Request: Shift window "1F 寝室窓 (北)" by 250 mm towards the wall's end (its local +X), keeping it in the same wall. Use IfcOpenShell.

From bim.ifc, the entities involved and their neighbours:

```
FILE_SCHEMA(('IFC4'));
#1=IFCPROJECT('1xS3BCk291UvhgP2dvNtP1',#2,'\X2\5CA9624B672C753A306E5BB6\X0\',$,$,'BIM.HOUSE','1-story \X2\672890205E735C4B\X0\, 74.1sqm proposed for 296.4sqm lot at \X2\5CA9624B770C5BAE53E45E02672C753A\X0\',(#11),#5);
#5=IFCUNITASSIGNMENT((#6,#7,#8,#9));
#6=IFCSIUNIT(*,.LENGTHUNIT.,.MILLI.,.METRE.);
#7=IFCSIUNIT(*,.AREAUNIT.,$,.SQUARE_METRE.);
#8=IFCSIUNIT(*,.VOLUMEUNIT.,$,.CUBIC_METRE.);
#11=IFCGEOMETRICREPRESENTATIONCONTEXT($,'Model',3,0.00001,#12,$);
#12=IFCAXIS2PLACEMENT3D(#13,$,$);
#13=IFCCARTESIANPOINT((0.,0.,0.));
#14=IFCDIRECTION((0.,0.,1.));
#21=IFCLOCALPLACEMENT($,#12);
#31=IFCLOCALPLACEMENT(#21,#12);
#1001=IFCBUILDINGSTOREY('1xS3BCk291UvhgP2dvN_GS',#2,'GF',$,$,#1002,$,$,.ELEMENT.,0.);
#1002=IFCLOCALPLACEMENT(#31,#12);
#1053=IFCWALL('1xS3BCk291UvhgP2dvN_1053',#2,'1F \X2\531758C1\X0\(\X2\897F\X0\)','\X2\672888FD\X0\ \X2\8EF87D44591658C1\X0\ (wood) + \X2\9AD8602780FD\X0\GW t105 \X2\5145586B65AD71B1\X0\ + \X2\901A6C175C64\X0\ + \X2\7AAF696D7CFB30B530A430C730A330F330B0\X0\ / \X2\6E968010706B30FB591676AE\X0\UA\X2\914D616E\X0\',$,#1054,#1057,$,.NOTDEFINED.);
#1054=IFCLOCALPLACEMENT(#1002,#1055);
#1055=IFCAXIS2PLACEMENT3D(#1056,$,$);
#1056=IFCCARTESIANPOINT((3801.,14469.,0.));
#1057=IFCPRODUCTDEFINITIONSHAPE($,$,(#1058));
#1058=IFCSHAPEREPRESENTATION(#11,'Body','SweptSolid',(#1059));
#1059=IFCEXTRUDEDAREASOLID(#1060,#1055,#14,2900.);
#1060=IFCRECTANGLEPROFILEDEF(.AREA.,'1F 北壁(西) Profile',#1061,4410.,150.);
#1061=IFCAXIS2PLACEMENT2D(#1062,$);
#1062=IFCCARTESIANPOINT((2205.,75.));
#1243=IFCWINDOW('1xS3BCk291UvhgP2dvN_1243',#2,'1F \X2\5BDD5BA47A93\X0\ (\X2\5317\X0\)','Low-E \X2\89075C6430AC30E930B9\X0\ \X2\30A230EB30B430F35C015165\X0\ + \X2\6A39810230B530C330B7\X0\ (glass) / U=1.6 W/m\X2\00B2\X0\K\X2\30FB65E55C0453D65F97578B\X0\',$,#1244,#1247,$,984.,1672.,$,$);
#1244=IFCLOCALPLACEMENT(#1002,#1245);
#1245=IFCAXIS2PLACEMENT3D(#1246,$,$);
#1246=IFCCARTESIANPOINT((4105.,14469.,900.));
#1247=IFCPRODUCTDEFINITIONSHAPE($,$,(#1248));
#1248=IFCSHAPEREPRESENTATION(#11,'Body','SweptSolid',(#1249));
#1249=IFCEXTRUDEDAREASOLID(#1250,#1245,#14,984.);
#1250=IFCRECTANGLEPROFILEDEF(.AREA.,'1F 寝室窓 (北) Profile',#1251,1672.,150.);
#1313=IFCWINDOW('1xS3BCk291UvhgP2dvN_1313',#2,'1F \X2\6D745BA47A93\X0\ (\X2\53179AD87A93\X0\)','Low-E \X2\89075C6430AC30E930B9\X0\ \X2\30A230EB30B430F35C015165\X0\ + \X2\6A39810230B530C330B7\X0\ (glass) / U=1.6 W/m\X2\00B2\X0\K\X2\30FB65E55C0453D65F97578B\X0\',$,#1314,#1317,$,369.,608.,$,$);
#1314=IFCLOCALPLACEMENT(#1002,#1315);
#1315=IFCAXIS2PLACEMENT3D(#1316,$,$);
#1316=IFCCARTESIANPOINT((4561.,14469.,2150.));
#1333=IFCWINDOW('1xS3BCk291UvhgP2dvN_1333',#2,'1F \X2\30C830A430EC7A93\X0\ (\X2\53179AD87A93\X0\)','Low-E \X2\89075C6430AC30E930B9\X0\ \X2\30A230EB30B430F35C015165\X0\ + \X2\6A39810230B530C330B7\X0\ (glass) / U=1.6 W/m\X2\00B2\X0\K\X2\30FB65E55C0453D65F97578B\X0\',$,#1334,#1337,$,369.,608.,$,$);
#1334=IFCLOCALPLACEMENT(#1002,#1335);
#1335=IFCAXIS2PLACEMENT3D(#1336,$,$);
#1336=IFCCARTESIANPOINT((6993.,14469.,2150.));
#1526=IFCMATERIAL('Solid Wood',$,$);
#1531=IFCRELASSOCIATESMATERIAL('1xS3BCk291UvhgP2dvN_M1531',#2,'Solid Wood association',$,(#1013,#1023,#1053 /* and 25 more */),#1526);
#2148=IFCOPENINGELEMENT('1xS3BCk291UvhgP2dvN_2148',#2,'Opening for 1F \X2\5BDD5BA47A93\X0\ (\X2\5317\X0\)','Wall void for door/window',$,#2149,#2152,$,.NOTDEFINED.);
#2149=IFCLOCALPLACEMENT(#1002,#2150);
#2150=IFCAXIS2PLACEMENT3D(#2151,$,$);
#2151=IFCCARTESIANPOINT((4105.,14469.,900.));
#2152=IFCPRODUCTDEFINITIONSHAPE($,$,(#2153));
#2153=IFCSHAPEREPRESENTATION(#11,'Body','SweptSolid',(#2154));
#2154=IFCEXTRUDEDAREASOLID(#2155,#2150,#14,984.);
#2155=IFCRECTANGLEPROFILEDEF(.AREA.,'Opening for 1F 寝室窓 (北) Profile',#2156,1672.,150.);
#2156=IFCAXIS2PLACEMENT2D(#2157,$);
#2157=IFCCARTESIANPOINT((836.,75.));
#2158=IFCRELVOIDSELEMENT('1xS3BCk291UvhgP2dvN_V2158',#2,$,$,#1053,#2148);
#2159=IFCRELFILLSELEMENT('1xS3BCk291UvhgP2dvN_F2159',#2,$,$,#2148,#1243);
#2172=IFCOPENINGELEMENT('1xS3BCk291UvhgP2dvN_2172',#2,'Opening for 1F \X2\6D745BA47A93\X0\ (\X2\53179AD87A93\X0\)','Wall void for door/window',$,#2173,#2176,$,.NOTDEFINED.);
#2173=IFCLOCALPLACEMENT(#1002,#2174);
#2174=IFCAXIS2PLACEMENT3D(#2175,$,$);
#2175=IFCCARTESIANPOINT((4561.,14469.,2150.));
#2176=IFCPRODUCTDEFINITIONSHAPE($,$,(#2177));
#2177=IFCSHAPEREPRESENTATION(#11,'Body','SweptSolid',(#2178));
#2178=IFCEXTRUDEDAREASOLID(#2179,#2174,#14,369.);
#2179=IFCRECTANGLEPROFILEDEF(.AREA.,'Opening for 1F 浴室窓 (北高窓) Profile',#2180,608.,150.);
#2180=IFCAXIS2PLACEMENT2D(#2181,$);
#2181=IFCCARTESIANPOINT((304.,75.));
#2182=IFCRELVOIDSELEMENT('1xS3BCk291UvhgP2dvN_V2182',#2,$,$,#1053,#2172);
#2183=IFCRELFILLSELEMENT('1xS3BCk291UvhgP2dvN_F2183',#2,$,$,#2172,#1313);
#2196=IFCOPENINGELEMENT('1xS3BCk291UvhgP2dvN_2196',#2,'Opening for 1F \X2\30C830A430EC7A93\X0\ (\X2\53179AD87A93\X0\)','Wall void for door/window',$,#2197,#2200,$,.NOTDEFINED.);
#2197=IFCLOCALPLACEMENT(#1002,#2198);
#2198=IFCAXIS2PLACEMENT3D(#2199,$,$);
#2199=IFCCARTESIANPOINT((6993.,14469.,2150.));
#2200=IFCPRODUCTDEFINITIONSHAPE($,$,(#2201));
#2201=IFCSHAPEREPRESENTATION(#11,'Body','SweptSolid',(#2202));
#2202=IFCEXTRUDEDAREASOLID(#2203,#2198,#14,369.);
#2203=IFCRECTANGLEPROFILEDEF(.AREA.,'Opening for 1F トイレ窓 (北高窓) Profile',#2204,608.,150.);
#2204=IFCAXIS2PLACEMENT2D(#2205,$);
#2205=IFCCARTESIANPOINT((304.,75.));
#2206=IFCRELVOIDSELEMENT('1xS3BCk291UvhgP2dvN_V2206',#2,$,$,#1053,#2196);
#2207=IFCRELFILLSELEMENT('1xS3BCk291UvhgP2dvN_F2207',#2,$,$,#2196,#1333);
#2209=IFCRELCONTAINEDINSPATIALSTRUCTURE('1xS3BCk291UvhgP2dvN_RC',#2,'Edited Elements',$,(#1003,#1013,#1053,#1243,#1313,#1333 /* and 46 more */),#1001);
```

```python
import ifcopenshell
import ifcopenshell.api.geometry
import ifcopenshell.util.placement
import ifcopenshell.util.unit

model = ifcopenshell.open("bim.ifc")
unit_scale = ifcopenshell.util.unit.calculate_unit_scale(model)

window = model.by_guid("1xS3BCk291UvhgP2dvN_1243")
opening = window.FillsVoids[0].RelatingOpeningElement
wall = opening.VoidsElements[0].RelatingBuildingElement

wall_matrix = ifcopenshell.util.placement.get_local_placement(wall.ObjectPlacement)
shift = wall_matrix[:3, 0] * 0.25 / unit_scale
before = ifcopenshell.util.placement.get_local_placement(window.ObjectPlacement)[:3, 3].copy()

# The window is not placed relative to its opening, so move both.
for product in (opening, window):
    matrix = ifcopenshell.util.placement.get_local_placement(product.ObjectPlacement)
    matrix[:3, 3] += shift
    ifcopenshell.api.geometry.edit_object_placement(model, product=product, matrix=matrix, is_si=False)

after = ifcopenshell.util.placement.get_local_placement(window.ObjectPlacement)[:3, 3]
print("window moved by", (after - before).round(3) + 0.0)

model.write("bim_updated.ifc")
```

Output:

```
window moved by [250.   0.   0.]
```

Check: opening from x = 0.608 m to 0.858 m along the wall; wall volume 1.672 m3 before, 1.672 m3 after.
